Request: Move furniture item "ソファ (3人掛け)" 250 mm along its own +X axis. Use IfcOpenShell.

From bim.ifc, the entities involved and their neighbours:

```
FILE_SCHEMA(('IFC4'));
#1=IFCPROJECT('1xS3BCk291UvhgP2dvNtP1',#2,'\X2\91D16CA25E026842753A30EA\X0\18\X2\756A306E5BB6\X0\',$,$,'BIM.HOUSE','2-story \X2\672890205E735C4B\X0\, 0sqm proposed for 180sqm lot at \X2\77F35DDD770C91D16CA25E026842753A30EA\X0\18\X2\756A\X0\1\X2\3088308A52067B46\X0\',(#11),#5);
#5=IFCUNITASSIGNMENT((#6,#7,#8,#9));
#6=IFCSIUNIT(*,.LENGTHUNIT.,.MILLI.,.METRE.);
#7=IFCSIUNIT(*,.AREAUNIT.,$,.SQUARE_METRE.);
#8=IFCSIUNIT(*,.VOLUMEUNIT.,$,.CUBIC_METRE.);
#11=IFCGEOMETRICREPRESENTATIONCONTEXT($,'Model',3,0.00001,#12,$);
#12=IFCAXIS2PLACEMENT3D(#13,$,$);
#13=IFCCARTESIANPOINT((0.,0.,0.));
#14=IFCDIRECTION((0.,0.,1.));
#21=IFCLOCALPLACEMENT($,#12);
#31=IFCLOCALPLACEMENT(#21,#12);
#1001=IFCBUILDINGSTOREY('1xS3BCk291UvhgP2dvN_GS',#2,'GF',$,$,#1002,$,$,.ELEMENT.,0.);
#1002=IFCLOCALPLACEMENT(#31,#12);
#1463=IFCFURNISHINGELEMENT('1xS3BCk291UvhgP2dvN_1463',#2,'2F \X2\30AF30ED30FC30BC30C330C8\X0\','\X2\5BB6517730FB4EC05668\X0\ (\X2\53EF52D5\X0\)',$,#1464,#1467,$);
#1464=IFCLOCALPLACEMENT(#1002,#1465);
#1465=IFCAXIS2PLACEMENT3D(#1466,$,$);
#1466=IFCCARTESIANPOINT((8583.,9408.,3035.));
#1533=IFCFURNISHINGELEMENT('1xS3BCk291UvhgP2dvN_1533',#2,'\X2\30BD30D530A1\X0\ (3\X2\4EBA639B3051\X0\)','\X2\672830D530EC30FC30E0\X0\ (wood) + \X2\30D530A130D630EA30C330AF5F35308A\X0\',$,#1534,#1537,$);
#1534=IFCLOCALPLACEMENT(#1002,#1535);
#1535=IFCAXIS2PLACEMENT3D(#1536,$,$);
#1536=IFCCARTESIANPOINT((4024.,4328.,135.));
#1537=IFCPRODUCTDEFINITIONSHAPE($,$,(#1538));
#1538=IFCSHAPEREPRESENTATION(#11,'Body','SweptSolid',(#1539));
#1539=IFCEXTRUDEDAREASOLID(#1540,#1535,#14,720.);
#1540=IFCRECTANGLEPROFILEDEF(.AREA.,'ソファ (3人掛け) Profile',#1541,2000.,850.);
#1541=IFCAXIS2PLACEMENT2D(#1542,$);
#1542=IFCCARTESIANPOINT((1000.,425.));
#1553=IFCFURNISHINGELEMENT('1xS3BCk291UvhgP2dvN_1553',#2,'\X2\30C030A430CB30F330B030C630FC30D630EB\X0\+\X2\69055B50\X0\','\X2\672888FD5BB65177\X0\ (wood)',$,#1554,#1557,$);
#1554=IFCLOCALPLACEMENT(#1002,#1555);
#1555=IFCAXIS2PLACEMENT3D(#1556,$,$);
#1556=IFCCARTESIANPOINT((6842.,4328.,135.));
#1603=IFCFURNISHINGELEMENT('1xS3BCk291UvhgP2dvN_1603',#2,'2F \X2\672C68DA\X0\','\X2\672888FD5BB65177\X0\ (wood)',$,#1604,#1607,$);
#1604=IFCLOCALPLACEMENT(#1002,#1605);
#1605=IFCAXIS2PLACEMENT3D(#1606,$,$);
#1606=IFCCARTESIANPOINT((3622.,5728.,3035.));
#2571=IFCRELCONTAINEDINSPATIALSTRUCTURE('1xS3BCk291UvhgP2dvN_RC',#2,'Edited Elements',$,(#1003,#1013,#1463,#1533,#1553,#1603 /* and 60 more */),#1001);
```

```python
import ifcopenshell
import ifcopenshell.api.geometry
import ifcopenshell.util.placement
import ifcopenshell.util.unit

model = ifcopenshell.open("bim.ifc")
unit_scale = ifcopenshell.util.unit.calculate_unit_scale(model)

item = model.by_guid("1xS3BCk291UvhgP2dvN_1533")
matrix = ifcopenshell.util.placement.get_local_placement(item.ObjectPlacement)
matrix[:3, 3] += matrix[:3, 0] * 0.25 / unit_scale
ifcopenshell.api.geometry.edit_object_placement(model, product=item, matrix=matrix, is_si=False)

print(ifcopenshell.util.placement.get_local_placement(item.ObjectPlacement).round(3) + 0.0)

model.write("bim-out.ifc")
```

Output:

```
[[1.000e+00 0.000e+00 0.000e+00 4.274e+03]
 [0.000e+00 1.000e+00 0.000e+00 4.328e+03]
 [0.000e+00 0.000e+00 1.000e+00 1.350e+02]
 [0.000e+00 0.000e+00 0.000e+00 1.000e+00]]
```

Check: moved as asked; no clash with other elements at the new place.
